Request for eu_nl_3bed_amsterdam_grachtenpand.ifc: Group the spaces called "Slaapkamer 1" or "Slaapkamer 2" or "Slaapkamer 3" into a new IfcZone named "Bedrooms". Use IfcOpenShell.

First a look at what the model holds.

```python
import ifcopenshell

model = ifcopenshell.open("eu_nl_3bed_amsterdam_grachtenpand.ifc")
print(model.schema)
seen = {}
for space in model.by_type("IfcSpace"):
    seen[space.LongName] = seen.get(space.LongName, 0) + 1
for name, count in sorted(seen.items(), key=str):
    print(count, "x", name)
print("zones:", [z.Name for z in model.by_type("IfcZone")][:20])
```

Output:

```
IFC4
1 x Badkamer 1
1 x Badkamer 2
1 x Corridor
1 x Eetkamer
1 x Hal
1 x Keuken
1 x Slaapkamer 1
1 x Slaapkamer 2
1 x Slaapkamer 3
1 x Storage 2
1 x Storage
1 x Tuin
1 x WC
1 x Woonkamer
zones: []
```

```python
import ifcopenshell
import ifcopenshell.api.group
import ifcopenshell.api.root

model = ifcopenshell.open("eu_nl_3bed_amsterdam_grachtenpand.ifc")

names = {"Slaapkamer 1", "Slaapkamer 2", "Slaapkamer 3"}
spaces = [s for s in model.by_type("IfcSpace") if s.LongName in names]

zone = ifcopenshell.api.root.create_entity(model, ifc_class="IfcZone", name="Bedrooms")
ifcopenshell.api.group.assign_group(model, products=spaces, group=zone)
print(len(spaces), "spaces in", zone.Name)

model.write("eu_nl_3bed_amsterdam_grachtenpand_edited.ifc")
```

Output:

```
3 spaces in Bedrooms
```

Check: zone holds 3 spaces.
